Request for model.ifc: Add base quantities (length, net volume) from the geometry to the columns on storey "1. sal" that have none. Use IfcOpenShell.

First a look at what the model holds.

```python
import ifcopenshell
import ifcopenshell.util.element
import ifcopenshell.util.unit

model = ifcopenshell.open("model.ifc")
print(model.schema)
for unit_type in ("LENGTHUNIT", "AREAUNIT", "VOLUMEUNIT"):
    print(unit_type, ifcopenshell.util.unit.calculate_unit_scale(model, unit_type))
storey = next(s for s in model.by_type("IfcBuildingStorey") if s.Name == "1. sal")
columns = [e for e in ifcopenshell.util.element.get_decomposition(storey) if e.is_a("IfcColumn")]
for e in sorted(columns, key=lambda e: e.id()):
    print(e.id(), e.is_a(), e.Name, list(ifcopenshell.util.element.get_psets(e, qtos_only=True)), sep=" | ")
```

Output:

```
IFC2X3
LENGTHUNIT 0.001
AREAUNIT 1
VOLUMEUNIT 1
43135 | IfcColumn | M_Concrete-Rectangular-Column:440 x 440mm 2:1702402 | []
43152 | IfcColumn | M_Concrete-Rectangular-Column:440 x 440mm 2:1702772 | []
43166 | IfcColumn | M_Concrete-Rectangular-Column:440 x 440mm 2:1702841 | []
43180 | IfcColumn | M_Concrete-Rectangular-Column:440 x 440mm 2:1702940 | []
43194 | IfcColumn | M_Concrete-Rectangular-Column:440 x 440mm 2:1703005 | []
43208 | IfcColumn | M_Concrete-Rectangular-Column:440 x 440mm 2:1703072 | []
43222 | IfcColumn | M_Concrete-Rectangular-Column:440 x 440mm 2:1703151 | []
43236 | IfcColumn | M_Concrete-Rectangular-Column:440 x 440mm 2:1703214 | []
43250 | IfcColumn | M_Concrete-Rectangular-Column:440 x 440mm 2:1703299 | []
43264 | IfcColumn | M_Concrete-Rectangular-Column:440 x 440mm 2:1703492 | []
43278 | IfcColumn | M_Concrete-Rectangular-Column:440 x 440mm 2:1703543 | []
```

```python
import ifcopenshell
import ifcopenshell.api.pset
import ifcopenshell.geom
import ifcopenshell.util.element
import ifcopenshell.util.shape
import ifcopenshell.util.unit

model = ifcopenshell.open("model.ifc")
unit_scale = ifcopenshell.util.unit.calculate_unit_scale(model)
volume_scale = ifcopenshell.util.unit.calculate_unit_scale(model, "VOLUMEUNIT")
settings = ifcopenshell.geom.settings()

storey = next(s for s in model.by_type("IfcBuildingStorey") if s.Name == "1. sal")
columns = [e for e in ifcopenshell.util.element.get_decomposition(storey) if e.is_a("IfcColumn")]

for e in sorted(columns, key=lambda e: e.id()):
    if ifcopenshell.util.element.get_psets(e, qtos_only=True, should_inherit=False):
        continue
    # Geometry comes back in metres, in the element's own axes.
    shape = ifcopenshell.geom.create_shape(settings, e)
    values = {
        "Length": ifcopenshell.util.shape.get_z(shape.geometry) / unit_scale,
        "NetVolume": ifcopenshell.util.shape.get_volume(shape.geometry) / volume_scale,
    }
    qto = ifcopenshell.api.pset.add_qto(model, product=e, name="BaseQuantities")
    ifcopenshell.api.pset.edit_qto(model, qto=qto, properties=values)
    print(e.id(), {k: round(v, 3) for k, v in values.items()})

model.write("model_updated.ifc")
```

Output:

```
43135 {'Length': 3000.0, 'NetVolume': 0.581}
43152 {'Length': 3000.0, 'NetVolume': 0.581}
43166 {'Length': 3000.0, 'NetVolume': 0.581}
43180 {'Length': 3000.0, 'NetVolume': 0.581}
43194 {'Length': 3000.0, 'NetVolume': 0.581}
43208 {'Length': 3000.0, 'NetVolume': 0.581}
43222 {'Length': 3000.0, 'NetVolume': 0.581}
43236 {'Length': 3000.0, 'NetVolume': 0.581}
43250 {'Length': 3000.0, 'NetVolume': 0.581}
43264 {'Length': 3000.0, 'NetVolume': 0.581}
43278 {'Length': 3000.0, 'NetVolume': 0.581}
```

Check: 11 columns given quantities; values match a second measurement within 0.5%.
